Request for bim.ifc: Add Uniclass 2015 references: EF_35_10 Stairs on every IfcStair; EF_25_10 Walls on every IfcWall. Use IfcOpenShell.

First a look at what the model holds.

```python
import ifcopenshell

model = ifcopenshell.open("bim.ifc")
print(model.schema)
print("classifications:", [c.Name for c in model.by_type("IfcClassification")])
for ifc_class in ("IfcDoor", "IfcRoof", "IfcStair", "IfcWall", "IfcWindow"):
    print(ifc_class, len(model.by_type(ifc_class)))
```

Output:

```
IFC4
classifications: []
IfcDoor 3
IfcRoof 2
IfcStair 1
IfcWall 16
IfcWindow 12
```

```python
import ifcopenshell
import ifcopenshell.api.classification

model = ifcopenshell.open("bim.ifc")

system = ifcopenshell.api.classification.add_classification(model, classification="Uniclass 2015")

codes = {
    "IfcStair": ("EF_35_10", "Stairs"),
    "IfcWall": ("EF_25_10", "Walls"),
}
for ifc_class, (code, name) in codes.items():
    products = model.by_type(ifc_class)
    ifcopenshell.api.classification.add_reference(
        model, products=products, classification=system, identification=code, name=name
    )
    print(code, len(products))

model.write("bim_v2.ifc")
```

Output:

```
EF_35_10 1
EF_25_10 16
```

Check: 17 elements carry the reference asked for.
